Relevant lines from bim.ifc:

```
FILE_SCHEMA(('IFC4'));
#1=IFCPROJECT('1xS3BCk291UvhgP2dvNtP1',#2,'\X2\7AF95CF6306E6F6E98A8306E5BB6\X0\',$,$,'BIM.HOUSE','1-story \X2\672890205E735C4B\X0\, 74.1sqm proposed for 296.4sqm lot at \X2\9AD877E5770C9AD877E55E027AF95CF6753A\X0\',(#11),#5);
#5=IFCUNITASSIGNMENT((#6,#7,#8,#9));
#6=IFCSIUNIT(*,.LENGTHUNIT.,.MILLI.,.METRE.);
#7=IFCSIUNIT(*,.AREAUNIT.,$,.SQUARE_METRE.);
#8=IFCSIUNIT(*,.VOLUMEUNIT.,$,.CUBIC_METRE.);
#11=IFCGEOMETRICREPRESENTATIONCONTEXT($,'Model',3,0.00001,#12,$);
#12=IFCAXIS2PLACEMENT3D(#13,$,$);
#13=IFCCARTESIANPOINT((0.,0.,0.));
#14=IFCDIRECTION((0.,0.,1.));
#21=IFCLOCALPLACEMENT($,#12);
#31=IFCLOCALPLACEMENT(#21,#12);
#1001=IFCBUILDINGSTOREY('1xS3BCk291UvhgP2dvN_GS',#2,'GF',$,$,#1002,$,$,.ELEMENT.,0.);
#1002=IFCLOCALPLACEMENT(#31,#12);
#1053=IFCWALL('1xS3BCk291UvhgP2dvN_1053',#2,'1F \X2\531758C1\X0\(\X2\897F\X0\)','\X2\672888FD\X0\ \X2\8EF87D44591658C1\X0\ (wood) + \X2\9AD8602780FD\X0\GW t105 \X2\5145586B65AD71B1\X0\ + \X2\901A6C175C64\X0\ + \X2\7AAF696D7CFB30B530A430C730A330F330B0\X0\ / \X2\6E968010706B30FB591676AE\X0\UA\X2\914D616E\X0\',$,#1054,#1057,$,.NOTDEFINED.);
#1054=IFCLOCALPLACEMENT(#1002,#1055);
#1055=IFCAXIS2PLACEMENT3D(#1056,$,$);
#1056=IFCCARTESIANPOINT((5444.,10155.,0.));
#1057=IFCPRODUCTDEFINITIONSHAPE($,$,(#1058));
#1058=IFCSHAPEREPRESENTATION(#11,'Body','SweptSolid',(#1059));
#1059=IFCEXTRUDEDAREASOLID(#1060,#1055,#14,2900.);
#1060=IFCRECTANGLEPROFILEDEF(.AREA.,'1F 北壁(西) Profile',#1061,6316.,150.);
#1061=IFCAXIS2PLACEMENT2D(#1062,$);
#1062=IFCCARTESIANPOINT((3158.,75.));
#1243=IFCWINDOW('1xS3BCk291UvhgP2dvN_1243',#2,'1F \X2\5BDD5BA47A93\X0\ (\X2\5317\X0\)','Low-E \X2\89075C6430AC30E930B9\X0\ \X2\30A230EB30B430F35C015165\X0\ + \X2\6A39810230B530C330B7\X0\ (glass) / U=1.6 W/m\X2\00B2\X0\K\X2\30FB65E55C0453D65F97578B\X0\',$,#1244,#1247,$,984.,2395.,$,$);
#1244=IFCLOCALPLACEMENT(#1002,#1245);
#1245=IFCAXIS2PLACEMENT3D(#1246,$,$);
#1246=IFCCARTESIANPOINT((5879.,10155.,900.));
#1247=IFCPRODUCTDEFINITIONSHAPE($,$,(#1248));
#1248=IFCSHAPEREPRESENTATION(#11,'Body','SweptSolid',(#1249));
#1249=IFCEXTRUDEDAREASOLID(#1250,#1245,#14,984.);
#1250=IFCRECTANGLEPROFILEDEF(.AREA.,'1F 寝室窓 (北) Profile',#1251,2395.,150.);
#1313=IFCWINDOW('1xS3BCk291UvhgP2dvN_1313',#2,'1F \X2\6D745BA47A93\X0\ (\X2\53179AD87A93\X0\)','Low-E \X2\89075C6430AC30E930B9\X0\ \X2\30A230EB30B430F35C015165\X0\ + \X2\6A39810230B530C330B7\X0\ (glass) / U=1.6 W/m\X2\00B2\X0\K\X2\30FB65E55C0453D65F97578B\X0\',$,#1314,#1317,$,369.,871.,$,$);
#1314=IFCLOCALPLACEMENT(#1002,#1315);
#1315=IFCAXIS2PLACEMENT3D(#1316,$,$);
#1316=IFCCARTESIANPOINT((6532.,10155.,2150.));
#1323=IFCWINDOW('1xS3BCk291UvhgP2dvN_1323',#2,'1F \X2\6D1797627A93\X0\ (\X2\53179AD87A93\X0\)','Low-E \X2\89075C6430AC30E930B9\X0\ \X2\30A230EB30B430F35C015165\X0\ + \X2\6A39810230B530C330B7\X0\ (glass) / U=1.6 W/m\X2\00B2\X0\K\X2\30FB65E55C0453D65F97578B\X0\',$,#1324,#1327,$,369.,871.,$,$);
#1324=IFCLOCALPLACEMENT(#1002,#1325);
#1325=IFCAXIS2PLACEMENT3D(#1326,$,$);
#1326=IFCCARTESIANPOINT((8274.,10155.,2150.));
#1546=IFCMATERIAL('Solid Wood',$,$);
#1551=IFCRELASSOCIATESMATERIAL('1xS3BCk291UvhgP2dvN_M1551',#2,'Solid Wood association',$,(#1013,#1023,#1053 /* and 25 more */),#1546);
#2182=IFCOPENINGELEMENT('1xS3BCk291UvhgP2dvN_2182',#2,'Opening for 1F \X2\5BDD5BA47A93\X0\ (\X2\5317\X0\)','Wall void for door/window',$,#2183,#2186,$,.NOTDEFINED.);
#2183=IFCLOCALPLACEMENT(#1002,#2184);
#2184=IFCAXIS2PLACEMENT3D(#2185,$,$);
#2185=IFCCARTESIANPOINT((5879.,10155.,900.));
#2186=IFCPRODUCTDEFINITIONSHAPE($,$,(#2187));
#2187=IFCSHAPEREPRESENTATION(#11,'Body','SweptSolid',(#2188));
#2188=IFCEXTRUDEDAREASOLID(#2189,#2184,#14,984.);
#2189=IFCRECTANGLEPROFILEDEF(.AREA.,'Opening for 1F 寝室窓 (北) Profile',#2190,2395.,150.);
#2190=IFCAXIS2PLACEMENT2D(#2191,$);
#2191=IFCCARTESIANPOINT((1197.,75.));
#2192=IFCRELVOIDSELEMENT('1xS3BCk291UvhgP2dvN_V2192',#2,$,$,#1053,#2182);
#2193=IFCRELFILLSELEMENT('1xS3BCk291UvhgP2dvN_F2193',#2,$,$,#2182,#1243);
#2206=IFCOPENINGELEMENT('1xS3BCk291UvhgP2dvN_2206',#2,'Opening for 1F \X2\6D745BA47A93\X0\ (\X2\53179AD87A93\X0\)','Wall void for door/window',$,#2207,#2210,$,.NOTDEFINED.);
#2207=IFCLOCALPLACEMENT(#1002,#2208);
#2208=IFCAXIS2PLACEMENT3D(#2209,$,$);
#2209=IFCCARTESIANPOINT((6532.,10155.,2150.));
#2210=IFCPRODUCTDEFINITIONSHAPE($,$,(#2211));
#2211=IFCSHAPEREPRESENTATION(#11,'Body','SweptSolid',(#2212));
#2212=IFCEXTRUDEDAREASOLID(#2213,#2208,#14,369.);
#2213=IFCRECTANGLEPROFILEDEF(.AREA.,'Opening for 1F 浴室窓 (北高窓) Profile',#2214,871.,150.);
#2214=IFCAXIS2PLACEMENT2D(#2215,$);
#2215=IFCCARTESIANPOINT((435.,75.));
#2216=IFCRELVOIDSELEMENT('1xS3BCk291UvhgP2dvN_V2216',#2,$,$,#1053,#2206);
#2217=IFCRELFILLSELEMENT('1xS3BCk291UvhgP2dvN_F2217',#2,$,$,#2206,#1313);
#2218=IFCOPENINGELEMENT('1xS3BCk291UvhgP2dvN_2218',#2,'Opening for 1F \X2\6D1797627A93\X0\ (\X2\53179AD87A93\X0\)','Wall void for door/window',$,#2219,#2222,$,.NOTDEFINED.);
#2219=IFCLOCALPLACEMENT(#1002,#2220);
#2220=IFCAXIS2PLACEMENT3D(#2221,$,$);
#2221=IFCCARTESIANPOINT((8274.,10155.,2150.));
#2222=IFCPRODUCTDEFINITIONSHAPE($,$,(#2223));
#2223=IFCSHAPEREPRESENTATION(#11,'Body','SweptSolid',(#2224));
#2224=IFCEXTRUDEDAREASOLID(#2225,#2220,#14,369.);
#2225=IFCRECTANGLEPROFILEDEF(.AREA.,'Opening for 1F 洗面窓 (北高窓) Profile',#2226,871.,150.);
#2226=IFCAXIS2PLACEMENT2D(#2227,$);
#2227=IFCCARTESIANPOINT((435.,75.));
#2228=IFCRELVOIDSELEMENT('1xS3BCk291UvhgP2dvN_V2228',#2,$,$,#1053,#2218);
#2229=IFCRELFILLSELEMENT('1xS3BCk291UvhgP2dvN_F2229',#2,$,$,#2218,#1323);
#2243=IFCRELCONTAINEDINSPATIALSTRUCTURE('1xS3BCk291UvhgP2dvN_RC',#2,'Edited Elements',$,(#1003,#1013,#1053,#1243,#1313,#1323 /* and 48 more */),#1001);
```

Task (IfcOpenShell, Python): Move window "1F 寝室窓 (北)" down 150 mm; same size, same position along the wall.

```python
import numpy as np
import ifcopenshell
import ifcopenshell.api.geometry
import ifcopenshell.util.placement
import ifcopenshell.util.unit

model = ifcopenshell.open("bim.ifc")
unit_scale = ifcopenshell.util.unit.calculate_unit_scale(model)

window = model.by_guid("1xS3BCk291UvhgP2dvN_1243")
opening = window.FillsVoids[0].RelatingOpeningElement
dz = -0.15 / unit_scale

shift = np.array([0.0, 0.0, dz])
# The window is not placed relative to its opening, so move both.
for product in (opening, window):
    matrix = ifcopenshell.util.placement.get_local_placement(product.ObjectPlacement)
    matrix[:3, 3] += shift
    ifcopenshell.api.geometry.edit_object_placement(model, product=product, matrix=matrix, is_si=False)

print(f"moved by {dz * unit_scale:+.3f} m")

model.write("bim_edited.ifc")
```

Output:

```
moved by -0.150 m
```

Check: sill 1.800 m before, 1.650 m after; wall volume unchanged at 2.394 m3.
